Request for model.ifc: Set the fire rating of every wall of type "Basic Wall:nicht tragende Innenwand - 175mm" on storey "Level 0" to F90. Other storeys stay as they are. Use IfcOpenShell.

First a look at what the model holds.

```python
import ifcopenshell
import ifcopenshell.util.element

model = ifcopenshell.open("model.ifc")
print(model.schema)
storey = next(s for s in model.by_type("IfcBuildingStorey") if s.Name == "Level 0")
walls = [e for e in ifcopenshell.util.element.get_decomposition(storey) if e.is_a("IfcWall")]
seen = {}
for e in walls:
    element_type = ifcopenshell.util.element.get_type(e)
    key = (element_type.Name if element_type != e and element_type else None, ifcopenshell.util.element.get_pset(e, "Pset_WallCommon", "FireRating"))
    seen[key] = seen.get(key, 0) + 1
for (name, value), count in sorted(seen.items(), key=str):
    print(count, "x", name, "|", value)
```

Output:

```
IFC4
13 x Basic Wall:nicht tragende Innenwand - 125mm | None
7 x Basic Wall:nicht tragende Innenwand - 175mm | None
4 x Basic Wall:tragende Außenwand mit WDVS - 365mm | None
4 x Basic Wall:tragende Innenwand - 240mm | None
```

```python
import ifcopenshell
import ifcopenshell.api.pset
import ifcopenshell.util.element

model = ifcopenshell.open("model.ifc")

storey = next(s for s in model.by_type("IfcBuildingStorey") if s.Name == "Level 0")
walls = [e for e in ifcopenshell.util.element.get_decomposition(storey) if e.is_a("IfcWall")]

count = 0
for e in walls:
    element_type = ifcopenshell.util.element.get_type(e)
    if element_type in (None, e) or element_type.Name != "Basic Wall:nicht tragende Innenwand - 175mm":
        continue
    # add_pset returns the element's existing set when there is one.
    pset = ifcopenshell.api.pset.add_pset(model, product=e, name="Pset_WallCommon")
    ifcopenshell.api.pset.edit_pset(model, pset=pset, properties={"FireRating": "F90"})
    count += 1

print(count, "walls updated")

model.write("model_updated.ifc")
```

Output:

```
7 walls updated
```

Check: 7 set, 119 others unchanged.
